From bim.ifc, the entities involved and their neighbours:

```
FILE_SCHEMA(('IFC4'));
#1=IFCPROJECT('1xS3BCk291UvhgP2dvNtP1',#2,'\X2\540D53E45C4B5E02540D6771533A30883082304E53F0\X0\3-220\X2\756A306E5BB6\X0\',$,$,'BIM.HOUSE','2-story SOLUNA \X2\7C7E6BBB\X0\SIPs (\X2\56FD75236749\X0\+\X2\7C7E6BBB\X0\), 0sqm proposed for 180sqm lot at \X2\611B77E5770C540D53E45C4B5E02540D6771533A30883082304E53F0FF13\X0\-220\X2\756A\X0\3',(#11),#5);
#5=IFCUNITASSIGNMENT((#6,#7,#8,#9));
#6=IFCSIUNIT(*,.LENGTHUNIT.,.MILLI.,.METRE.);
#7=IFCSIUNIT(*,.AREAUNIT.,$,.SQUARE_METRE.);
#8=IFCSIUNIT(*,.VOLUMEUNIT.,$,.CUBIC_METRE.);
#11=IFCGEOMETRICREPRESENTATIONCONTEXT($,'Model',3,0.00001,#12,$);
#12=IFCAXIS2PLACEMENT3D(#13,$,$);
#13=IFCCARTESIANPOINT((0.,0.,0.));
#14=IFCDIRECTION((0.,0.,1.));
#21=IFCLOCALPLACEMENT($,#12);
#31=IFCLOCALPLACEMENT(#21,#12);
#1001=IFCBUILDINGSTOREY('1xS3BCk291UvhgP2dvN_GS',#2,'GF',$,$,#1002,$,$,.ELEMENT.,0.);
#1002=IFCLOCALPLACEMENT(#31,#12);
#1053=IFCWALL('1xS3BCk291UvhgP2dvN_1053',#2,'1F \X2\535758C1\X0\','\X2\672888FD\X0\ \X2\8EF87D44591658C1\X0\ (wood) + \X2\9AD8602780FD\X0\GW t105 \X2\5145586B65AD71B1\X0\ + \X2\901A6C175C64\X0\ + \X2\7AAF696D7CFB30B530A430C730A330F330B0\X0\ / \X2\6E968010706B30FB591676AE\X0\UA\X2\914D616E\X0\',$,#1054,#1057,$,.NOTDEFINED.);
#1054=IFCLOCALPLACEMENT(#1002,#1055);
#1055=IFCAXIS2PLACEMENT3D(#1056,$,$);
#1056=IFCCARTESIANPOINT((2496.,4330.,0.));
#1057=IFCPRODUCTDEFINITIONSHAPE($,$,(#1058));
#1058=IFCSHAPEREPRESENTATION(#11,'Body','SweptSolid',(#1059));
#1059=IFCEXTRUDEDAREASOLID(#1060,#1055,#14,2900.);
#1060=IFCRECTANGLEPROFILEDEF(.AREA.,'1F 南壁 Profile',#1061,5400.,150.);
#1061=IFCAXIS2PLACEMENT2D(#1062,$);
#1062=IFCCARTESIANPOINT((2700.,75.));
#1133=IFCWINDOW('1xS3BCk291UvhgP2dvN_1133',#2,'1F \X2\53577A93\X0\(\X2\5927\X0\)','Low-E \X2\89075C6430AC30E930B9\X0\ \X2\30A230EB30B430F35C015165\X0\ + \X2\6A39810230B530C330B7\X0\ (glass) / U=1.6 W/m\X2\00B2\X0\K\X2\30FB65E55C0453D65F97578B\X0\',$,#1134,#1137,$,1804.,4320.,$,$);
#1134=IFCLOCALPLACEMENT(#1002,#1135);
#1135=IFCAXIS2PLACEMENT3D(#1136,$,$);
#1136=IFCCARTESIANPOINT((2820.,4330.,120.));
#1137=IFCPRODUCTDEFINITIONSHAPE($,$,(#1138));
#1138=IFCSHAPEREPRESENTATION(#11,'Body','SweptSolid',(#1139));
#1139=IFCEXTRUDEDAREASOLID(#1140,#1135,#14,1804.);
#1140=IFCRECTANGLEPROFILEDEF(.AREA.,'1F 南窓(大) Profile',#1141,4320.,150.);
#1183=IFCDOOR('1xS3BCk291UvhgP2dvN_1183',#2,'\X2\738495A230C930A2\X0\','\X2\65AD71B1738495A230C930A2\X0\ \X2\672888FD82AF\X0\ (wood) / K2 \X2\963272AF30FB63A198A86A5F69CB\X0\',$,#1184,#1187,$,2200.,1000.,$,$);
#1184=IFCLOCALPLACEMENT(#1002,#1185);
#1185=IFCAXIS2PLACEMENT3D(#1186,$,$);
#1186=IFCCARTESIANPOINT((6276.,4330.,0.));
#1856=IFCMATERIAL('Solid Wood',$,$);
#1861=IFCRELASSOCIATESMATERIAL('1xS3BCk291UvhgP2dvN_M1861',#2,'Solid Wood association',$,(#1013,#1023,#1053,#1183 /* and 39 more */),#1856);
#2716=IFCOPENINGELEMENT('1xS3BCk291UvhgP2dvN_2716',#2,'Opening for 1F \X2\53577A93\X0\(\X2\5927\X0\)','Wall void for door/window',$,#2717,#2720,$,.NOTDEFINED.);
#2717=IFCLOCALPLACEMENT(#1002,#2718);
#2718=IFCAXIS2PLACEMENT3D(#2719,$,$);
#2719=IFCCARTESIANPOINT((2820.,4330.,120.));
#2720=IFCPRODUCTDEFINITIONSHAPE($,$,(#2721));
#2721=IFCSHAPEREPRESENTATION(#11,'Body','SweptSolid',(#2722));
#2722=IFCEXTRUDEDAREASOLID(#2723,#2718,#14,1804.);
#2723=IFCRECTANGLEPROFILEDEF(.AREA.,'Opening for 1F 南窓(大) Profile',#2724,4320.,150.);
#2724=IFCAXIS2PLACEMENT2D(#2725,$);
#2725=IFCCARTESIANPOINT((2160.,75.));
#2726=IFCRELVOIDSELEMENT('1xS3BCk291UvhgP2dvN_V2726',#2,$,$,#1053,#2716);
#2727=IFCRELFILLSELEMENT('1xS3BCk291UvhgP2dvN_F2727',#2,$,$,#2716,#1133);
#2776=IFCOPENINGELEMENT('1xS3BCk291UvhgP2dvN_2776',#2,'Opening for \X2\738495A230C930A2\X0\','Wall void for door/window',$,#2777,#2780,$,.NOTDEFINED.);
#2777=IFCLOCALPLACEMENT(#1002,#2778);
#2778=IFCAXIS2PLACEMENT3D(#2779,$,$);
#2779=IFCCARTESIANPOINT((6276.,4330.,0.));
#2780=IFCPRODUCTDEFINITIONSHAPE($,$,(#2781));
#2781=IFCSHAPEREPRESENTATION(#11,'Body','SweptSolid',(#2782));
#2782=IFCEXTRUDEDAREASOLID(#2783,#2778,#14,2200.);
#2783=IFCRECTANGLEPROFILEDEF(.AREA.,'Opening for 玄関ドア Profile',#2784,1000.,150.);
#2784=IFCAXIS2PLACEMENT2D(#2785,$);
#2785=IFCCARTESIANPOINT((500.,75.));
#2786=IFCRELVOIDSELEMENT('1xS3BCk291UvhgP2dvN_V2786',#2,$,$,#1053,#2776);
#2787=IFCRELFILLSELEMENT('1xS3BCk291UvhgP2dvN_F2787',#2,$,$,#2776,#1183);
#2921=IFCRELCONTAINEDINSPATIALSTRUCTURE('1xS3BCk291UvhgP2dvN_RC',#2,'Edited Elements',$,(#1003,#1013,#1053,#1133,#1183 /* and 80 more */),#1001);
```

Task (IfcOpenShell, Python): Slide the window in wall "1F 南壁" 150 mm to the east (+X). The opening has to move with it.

```python
import ifcopenshell
import ifcopenshell.api.geometry
import ifcopenshell.util.placement

model = ifcopenshell.open("bim.ifc")

window = model.by_guid("1xS3BCk291UvhgP2dvN_1133")
opening = window.FillsVoids[0].RelatingOpeningElement
wall = opening.VoidsElements[0].RelatingBuildingElement

wall_matrix = ifcopenshell.util.placement.get_local_placement(wall.ObjectPlacement)
shift = wall_matrix[:3, 0] * 150.0
before = ifcopenshell.util.placement.get_local_placement(window.ObjectPlacement)[:3, 3].copy()

# The window is not placed relative to its opening, so move both.
for product in (opening, window):
    matrix = ifcopenshell.util.placement.get_local_placement(product.ObjectPlacement)
    matrix[:3, 3] += shift
    ifcopenshell.api.geometry.edit_object_placement(model, product=product, matrix=matrix, is_si=False)

after = ifcopenshell.util.placement.get_local_placement(window.ObjectPlacement)[:3, 3]
print("window moved by", (after - before).round(3) + 0.0)

model.write("bim_v2.ifc")
```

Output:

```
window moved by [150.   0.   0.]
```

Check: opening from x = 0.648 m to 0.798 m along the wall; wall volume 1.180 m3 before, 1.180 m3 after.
